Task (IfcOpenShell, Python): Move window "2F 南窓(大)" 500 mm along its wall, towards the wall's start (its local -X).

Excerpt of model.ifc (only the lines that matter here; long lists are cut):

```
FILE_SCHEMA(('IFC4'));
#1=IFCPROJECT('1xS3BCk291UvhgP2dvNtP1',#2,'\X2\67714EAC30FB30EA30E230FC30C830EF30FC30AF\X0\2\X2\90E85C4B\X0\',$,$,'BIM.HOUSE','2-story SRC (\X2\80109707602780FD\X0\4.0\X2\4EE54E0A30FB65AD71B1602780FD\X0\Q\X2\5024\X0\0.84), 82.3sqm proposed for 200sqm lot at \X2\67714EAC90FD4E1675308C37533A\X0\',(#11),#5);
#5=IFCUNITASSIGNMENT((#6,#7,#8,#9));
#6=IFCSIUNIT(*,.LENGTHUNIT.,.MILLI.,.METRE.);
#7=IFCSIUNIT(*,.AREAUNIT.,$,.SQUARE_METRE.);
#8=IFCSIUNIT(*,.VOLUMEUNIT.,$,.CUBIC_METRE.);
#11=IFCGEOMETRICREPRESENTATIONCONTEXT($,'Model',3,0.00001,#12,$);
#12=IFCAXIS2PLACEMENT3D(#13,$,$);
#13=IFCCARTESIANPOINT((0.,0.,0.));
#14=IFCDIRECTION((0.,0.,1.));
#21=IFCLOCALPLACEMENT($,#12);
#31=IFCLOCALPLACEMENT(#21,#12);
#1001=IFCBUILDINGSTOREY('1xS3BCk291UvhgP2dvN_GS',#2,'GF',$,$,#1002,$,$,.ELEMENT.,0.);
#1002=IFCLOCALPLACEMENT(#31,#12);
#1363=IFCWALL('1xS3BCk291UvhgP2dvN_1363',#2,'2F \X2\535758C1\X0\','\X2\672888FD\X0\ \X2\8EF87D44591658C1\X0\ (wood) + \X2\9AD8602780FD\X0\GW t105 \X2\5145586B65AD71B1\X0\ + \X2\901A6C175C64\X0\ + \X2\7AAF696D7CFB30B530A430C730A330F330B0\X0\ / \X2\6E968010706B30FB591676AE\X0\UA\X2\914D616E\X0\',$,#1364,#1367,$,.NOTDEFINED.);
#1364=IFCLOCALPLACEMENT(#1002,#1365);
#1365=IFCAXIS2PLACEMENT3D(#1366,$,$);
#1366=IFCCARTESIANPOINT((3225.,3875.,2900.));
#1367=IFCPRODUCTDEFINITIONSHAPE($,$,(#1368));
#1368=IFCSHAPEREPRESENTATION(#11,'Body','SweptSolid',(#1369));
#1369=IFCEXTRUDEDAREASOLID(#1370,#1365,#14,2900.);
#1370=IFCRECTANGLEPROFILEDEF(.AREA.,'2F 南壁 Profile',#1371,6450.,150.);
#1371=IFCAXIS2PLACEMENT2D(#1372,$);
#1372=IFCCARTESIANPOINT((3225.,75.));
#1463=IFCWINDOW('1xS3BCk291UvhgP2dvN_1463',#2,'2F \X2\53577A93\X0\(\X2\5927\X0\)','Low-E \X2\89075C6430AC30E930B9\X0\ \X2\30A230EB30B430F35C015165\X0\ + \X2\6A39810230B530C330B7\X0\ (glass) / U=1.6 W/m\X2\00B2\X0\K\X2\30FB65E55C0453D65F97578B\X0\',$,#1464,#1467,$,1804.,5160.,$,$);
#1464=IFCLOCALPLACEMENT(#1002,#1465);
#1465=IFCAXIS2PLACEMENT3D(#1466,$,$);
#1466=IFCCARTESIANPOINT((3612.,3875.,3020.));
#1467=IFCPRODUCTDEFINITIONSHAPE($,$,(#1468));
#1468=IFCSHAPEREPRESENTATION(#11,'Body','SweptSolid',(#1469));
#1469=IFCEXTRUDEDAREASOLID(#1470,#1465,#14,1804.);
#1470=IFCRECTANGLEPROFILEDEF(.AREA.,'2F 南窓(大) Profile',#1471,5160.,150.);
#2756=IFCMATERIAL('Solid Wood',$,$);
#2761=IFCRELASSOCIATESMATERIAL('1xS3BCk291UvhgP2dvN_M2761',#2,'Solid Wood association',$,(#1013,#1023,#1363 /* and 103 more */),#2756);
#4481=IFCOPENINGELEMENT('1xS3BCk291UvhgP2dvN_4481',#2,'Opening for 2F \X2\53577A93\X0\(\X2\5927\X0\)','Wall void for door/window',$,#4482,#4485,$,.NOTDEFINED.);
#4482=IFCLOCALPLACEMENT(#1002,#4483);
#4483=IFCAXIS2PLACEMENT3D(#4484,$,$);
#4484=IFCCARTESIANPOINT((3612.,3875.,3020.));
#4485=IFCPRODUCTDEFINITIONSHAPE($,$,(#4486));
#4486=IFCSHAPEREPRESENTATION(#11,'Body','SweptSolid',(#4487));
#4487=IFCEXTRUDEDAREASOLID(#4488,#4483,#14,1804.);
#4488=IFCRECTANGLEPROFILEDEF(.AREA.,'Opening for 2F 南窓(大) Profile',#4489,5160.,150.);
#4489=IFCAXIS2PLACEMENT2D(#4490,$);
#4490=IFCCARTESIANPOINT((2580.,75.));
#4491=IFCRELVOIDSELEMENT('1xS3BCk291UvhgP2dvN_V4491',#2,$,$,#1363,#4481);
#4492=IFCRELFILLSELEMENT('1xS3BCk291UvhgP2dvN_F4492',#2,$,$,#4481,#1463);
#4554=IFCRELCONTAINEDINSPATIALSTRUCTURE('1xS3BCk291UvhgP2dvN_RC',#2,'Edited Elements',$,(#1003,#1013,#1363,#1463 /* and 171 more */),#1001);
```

```python
import ifcopenshell
import ifcopenshell.api.geometry
import ifcopenshell.util.placement
import ifcopenshell.util.unit

model = ifcopenshell.open("model.ifc")
unit_scale = ifcopenshell.util.unit.calculate_unit_scale(model)

window = model.by_id(1463)
opening = window.FillsVoids[0].RelatingOpeningElement
wall = opening.VoidsElements[0].RelatingBuildingElement

wall_matrix = ifcopenshell.util.placement.get_local_placement(wall.ObjectPlacement)
shift = wall_matrix[:3, 0] * -0.5 / unit_scale
before = ifcopenshell.util.placement.get_local_placement(window.ObjectPlacement)[:3, 3].copy()

# The window is not placed relative to its opening, so move both.
for product in (opening, window):
    matrix = ifcopenshell.util.placement.get_local_placement(product.ObjectPlacement)
    matrix[:3, 3] += shift
    ifcopenshell.api.geometry.edit_object_placement(model, product=product, matrix=matrix, is_si=False)

after = ifcopenshell.util.placement.get_local_placement(window.ObjectPlacement)[:3, 3]
print("window moved by", (after - before).round(3) + 0.0)

model.write("model-out.ifc")
```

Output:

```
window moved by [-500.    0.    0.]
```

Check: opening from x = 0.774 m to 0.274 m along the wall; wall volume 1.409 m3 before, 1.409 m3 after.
